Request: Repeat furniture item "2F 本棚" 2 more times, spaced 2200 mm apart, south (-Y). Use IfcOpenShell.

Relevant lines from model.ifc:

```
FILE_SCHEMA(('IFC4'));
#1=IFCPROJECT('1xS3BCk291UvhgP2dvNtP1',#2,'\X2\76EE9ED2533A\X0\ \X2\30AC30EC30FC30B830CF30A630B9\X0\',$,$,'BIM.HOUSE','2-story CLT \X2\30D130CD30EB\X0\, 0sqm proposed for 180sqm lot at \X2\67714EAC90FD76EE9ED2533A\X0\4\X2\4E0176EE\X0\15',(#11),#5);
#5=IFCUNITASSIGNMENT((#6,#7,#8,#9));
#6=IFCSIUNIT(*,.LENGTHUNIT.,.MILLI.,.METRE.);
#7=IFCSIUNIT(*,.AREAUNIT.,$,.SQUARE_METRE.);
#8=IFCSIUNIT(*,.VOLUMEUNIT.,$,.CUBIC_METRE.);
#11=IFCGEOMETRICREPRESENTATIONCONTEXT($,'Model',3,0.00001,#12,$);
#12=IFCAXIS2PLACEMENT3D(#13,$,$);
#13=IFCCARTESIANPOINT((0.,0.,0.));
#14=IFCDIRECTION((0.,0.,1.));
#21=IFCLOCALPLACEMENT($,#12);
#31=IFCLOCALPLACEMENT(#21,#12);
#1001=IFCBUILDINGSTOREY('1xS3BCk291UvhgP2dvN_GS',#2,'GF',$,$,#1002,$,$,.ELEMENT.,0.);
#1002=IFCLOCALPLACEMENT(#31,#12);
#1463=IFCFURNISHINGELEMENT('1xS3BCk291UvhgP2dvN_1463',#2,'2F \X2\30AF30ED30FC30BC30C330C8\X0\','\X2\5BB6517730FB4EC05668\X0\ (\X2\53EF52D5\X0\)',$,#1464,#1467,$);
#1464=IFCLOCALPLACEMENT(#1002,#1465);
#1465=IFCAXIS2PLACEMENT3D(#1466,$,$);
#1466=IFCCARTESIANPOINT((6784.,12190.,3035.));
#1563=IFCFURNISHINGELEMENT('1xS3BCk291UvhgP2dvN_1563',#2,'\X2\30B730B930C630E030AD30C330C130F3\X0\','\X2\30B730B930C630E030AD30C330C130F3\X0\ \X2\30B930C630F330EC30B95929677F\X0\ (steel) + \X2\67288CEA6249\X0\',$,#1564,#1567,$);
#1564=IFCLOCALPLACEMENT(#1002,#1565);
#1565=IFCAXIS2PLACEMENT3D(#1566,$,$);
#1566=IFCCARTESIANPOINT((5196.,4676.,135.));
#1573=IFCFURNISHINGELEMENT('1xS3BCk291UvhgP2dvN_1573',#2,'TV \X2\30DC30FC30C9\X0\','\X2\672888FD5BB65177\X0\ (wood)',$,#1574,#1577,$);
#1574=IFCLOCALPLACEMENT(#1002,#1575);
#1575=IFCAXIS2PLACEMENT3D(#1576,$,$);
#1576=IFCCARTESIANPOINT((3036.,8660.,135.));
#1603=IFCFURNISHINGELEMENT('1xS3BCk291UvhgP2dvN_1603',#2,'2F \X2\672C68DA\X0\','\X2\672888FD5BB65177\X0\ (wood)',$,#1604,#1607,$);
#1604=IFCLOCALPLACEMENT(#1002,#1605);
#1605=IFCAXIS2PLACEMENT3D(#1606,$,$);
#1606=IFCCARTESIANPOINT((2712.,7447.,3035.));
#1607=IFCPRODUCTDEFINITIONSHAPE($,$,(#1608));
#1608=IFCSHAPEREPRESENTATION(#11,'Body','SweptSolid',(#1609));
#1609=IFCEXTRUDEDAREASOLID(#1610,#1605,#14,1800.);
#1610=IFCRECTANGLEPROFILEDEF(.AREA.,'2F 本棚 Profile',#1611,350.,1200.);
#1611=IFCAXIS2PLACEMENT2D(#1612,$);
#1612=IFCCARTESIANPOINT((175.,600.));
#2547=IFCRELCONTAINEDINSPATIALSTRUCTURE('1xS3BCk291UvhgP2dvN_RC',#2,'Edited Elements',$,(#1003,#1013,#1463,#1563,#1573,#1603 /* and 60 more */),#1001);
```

```python
import numpy as np
import ifcopenshell
import ifcopenshell.api.geometry
import ifcopenshell.api.root
import ifcopenshell.util.element
import ifcopenshell.util.placement
import ifcopenshell.util.unit

model = ifcopenshell.open("model.ifc")
unit_scale = ifcopenshell.util.unit.calculate_unit_scale(model)


def reuse_history(source, copy):
    """copy_class also copies each property set's owner history, people and application; keep the originals."""
    for rel in copy.IsDefinedBy:
        if rel.is_a("IfcRelDefinesByProperties") and (history := rel.RelatingPropertyDefinition.OwnerHistory):
            rel.RelatingPropertyDefinition.OwnerHistory = source.OwnerHistory
            ifcopenshell.util.element.remove_deep2(model, history)


source = model.by_guid("1xS3BCk291UvhgP2dvN_1603")
base = ifcopenshell.util.placement.get_local_placement(source.ObjectPlacement)
step = np.array([0.0, -1.0, 0.0]) * 2.2 / unit_scale

for i in range(1, 3):
    copy = ifcopenshell.api.root.copy_class(model, product=source)
    copy.Representation = ifcopenshell.util.element.copy_deep(
        model, source.Representation, exclude=["IfcGeometricRepresentationContext", "IfcRepresentationMap"]
    )
    reuse_history(source, copy)
    matrix = base.copy()
    matrix[:3, 3] += i * step
    print("added at", matrix[:3, 3].round(3) + 0.0)
    ifcopenshell.api.geometry.edit_object_placement(model, product=copy, matrix=matrix, is_si=False)

model.write("model_updated.ifc")
```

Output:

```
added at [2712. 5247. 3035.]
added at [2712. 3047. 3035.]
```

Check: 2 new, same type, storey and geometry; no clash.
